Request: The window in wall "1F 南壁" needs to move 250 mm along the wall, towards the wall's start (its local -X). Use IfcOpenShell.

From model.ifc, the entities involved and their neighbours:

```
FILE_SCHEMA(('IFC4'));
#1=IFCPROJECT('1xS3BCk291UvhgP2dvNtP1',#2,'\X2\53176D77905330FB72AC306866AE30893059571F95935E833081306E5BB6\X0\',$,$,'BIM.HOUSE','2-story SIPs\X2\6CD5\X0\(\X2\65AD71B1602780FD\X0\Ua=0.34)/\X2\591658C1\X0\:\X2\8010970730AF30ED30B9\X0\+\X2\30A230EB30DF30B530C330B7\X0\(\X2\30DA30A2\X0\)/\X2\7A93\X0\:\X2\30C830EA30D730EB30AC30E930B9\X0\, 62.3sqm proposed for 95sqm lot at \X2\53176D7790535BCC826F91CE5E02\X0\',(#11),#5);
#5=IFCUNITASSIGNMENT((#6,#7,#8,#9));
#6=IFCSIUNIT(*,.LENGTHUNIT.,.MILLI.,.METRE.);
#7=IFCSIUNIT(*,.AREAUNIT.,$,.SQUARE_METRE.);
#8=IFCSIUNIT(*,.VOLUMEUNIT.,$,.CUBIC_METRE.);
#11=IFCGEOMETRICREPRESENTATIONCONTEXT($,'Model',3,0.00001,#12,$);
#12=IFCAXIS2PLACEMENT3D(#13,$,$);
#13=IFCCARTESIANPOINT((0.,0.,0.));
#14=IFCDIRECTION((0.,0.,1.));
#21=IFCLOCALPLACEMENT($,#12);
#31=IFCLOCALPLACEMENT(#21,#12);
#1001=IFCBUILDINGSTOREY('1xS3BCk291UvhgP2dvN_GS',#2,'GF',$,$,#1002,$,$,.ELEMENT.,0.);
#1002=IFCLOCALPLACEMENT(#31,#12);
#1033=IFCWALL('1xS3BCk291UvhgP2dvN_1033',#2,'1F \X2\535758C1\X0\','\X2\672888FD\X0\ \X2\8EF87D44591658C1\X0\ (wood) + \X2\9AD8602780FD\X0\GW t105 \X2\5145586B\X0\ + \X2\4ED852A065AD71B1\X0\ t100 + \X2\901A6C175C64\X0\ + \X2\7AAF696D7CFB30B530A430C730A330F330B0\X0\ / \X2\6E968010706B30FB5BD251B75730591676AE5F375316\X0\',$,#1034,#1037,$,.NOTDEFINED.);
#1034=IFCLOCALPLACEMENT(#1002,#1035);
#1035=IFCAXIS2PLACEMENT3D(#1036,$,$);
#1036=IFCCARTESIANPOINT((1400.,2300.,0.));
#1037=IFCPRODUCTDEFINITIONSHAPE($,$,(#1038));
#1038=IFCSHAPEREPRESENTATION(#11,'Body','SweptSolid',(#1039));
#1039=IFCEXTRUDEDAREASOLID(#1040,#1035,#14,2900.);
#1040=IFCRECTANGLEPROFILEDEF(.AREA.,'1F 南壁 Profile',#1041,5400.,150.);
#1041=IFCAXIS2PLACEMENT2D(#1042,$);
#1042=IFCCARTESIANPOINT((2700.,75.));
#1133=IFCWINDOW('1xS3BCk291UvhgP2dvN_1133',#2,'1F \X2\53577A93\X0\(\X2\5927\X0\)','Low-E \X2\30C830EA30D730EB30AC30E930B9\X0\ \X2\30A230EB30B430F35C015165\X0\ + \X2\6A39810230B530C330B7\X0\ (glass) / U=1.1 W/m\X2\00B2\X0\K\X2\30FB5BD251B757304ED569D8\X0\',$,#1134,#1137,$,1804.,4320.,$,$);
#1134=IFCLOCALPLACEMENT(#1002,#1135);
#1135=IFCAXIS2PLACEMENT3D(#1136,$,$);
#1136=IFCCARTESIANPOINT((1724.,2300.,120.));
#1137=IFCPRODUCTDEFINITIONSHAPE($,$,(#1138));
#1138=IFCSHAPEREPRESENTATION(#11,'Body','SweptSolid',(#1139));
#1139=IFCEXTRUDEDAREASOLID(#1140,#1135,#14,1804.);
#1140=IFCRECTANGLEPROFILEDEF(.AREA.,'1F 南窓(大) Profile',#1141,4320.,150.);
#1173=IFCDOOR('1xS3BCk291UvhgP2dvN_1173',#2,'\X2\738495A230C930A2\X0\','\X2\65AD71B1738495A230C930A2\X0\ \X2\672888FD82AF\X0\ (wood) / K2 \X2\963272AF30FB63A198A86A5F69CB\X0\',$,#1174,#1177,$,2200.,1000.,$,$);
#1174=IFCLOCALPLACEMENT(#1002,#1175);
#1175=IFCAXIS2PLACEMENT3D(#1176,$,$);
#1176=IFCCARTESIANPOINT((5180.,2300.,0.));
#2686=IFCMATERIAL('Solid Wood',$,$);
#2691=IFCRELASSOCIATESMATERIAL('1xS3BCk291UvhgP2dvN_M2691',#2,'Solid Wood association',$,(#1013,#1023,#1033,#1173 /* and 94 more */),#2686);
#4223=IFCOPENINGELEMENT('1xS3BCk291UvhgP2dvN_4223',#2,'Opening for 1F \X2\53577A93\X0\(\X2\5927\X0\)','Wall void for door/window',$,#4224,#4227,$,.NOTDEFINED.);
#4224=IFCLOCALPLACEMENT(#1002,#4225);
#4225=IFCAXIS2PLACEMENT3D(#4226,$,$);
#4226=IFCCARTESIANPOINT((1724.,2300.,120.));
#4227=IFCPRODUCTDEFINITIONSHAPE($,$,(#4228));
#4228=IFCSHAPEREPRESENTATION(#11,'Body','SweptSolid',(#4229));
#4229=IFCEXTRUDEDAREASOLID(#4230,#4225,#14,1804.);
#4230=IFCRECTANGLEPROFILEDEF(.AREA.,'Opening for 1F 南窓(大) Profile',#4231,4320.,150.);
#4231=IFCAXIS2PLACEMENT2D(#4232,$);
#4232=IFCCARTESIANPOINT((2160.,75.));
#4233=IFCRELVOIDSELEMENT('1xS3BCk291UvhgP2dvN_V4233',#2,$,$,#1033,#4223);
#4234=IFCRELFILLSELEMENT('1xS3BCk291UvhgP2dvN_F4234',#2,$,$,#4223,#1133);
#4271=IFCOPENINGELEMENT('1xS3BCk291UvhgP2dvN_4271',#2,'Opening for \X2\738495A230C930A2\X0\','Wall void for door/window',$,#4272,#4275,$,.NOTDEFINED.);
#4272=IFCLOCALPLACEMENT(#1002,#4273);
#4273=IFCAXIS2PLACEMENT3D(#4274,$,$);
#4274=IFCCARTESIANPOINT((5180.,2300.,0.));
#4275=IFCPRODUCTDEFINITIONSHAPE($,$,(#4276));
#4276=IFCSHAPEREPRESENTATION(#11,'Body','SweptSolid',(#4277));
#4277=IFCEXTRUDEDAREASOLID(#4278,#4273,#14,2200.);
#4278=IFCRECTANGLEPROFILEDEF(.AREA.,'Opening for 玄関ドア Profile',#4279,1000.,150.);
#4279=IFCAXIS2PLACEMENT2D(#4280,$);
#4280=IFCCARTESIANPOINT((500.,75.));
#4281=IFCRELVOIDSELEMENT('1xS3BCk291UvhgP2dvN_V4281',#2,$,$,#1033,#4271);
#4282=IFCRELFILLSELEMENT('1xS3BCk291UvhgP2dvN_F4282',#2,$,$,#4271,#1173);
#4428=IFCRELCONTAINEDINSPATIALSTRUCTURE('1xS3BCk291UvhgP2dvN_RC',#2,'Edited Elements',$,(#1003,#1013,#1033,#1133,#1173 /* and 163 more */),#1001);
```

```python
import ifcopenshell
import ifcopenshell.api.geometry
import ifcopenshell.util.placement
import ifcopenshell.util.unit

model = ifcopenshell.open("model.ifc")
unit_scale = ifcopenshell.util.unit.calculate_unit_scale(model)

window = model.by_guid("1xS3BCk291UvhgP2dvN_1133")
opening = window.FillsVoids[0].RelatingOpeningElement
wall = opening.VoidsElements[0].RelatingBuildingElement

wall_matrix = ifcopenshell.util.placement.get_local_placement(wall.ObjectPlacement)
shift = wall_matrix[:3, 0] * -0.25 / unit_scale
before = ifcopenshell.util.placement.get_local_placement(window.ObjectPlacement)[:3, 3].copy()

# The window is not placed relative to its opening, so move both.
for product in (opening, window):
    matrix = ifcopenshell.util.placement.get_local_placement(product.ObjectPlacement)
    matrix[:3, 3] += shift
    ifcopenshell.api.geometry.edit_object_placement(model, product=product, matrix=matrix, is_si=False)

after = ifcopenshell.util.placement.get_local_placement(window.ObjectPlacement)[:3, 3]
print("window moved by", (after - before).round(3) + 0.0)

model.write("model_rev.ifc")
```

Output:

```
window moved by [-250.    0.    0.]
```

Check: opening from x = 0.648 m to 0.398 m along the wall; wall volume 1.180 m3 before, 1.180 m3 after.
